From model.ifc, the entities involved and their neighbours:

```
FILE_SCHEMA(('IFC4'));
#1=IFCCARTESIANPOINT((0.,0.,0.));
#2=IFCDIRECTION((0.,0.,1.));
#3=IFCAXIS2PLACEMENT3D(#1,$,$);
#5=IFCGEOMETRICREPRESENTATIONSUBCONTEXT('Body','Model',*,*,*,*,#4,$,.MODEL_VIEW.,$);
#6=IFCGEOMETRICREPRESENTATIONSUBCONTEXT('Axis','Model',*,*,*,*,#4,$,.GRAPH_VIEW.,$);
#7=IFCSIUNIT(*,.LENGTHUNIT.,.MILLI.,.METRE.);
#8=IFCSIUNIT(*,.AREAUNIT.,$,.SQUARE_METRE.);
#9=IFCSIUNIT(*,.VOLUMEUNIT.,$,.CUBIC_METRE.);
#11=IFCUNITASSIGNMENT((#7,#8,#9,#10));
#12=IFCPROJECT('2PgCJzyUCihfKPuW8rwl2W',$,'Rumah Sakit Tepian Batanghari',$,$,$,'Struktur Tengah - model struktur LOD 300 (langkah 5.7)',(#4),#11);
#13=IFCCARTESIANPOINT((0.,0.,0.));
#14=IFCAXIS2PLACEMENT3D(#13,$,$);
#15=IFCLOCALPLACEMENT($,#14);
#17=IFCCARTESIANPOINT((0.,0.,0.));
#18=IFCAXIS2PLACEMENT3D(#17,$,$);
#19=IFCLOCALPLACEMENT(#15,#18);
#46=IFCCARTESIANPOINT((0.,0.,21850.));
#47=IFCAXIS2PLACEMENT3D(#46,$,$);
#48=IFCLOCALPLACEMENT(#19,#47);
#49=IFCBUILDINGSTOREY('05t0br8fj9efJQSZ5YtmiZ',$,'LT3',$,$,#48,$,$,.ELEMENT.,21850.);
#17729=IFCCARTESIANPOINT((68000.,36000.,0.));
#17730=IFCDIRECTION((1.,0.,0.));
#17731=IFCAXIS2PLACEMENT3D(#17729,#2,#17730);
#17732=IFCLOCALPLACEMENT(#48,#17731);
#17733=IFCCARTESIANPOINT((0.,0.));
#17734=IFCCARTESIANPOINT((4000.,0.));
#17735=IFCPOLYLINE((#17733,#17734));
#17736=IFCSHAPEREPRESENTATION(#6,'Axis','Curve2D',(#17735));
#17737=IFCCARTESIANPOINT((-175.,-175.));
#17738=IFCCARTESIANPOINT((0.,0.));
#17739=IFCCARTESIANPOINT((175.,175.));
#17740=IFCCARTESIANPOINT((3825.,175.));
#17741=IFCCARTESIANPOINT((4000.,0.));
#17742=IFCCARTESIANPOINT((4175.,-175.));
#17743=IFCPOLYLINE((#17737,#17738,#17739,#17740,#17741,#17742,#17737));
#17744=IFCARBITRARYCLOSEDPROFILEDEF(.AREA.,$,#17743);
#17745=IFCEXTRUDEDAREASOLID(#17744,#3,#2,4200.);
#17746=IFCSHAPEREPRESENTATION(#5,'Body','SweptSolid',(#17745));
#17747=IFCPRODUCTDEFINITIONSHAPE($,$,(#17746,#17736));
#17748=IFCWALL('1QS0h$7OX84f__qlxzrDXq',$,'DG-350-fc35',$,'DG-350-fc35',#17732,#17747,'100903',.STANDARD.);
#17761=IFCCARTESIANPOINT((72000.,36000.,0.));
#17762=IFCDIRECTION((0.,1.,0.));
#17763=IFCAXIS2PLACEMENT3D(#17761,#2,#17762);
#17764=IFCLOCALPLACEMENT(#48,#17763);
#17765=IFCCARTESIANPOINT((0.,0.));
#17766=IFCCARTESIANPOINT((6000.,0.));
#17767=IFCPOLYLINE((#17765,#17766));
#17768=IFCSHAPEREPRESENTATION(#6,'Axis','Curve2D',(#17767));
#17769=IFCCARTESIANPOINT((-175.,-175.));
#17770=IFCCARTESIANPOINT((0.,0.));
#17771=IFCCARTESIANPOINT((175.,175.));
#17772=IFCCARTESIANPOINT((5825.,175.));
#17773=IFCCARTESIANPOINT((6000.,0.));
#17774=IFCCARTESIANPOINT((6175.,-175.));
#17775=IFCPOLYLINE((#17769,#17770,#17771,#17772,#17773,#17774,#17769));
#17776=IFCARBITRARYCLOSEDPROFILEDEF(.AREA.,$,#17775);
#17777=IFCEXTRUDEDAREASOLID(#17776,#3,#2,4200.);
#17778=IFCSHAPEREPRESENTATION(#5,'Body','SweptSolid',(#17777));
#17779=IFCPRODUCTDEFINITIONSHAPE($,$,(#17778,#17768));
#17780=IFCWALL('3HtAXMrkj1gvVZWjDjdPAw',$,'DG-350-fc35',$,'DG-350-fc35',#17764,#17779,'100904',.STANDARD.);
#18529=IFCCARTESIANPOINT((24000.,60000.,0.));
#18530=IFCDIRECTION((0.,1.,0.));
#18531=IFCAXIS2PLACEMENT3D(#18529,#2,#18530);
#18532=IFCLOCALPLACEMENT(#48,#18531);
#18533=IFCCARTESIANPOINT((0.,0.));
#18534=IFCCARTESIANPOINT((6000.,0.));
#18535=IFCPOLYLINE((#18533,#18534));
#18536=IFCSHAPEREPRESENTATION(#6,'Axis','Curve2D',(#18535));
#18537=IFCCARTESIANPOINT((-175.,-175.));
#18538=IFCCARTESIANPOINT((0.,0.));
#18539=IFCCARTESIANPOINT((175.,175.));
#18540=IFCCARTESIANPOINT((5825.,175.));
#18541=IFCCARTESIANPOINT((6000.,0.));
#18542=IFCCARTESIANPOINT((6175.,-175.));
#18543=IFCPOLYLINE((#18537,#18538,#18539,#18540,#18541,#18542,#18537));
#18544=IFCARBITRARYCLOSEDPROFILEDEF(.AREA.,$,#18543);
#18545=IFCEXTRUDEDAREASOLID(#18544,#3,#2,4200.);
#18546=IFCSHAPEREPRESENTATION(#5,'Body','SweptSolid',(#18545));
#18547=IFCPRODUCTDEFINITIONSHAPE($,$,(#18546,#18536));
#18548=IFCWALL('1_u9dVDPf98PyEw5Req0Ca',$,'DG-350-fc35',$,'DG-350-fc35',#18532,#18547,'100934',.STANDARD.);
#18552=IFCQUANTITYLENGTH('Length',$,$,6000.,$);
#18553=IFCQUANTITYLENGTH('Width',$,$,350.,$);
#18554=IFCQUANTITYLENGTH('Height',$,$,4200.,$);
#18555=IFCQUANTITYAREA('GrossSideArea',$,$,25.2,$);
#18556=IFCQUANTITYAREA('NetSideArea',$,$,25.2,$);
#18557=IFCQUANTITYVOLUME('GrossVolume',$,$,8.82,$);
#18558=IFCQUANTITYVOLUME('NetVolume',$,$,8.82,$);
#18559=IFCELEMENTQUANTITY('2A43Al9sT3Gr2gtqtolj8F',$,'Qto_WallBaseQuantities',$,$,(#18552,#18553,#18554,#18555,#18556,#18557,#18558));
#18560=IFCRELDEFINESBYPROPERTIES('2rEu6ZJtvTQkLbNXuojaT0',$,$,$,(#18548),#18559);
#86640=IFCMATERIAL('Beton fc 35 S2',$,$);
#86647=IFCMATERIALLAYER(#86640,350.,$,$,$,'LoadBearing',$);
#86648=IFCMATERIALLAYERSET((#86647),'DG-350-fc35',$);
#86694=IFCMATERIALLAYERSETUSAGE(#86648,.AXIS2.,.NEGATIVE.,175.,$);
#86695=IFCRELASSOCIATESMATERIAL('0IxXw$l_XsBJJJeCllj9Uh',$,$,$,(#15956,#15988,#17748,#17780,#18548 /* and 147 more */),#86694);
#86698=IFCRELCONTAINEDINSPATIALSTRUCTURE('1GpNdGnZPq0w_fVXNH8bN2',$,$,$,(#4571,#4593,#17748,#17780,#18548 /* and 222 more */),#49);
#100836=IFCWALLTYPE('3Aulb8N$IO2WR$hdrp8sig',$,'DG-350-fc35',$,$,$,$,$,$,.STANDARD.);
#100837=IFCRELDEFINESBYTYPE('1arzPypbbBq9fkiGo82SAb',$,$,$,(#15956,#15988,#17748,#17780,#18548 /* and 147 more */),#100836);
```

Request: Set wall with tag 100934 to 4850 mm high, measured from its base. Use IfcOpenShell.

```python
import ifcopenshell
import ifcopenshell.api.pset
import ifcopenshell.geom
import ifcopenshell.util.element
import ifcopenshell.util.representation
import ifcopenshell.util.shape
import ifcopenshell.util.unit

model = ifcopenshell.open("model.ifc")
unit_scale = ifcopenshell.util.unit.calculate_unit_scale(model)
area_scale = ifcopenshell.util.unit.calculate_unit_scale(model, "AREAUNIT")
volume_scale = ifcopenshell.util.unit.calculate_unit_scale(model, "VOLUMEUNIT")
settings = ifcopenshell.geom.settings()


def volume(element):
    """Net volume in cubic metres, openings subtracted."""
    shape = ifcopenshell.geom.create_shape(settings, element)
    return ifcopenshell.util.shape.get_volume(shape.geometry)


wall = model.by_guid("1_u9dVDPf98PyEw5Req0Ca")
before = volume(wall)

body = ifcopenshell.util.representation.get_representation(wall, "Model", "Body")
solid = body.Items[0]
old_height = solid.Depth
solid.Depth = 4850.0
after = volume(wall)
thickness = 0.35  # wall thickness in metres

# Update the stored height, areas and volumes.
qto = model.by_id(ifcopenshell.util.element.get_pset(wall, "Qto_WallBaseQuantities", should_inherit=False)["id"])
ifcopenshell.api.pset.edit_qto(model, qto=qto, properties={
    "Height": solid.Depth,
    "GrossSideArea": ifcopenshell.util.element.get_pset(wall, "Qto_WallBaseQuantities", "GrossSideArea") * solid.Depth / old_height,
    "NetSideArea": after / thickness / area_scale,
    "GrossVolume": ifcopenshell.util.element.get_pset(wall, "Qto_WallBaseQuantities", "GrossVolume") * solid.Depth / old_height,
    "NetVolume": after / volume_scale,
})

print(f"height {old_height:g} -> {solid.Depth:g}, volume {before:.3f} -> {after:.3f} m3")

model.write("model-out.ifc")
```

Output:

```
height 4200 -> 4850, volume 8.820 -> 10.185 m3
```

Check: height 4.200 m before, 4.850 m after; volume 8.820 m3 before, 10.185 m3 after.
